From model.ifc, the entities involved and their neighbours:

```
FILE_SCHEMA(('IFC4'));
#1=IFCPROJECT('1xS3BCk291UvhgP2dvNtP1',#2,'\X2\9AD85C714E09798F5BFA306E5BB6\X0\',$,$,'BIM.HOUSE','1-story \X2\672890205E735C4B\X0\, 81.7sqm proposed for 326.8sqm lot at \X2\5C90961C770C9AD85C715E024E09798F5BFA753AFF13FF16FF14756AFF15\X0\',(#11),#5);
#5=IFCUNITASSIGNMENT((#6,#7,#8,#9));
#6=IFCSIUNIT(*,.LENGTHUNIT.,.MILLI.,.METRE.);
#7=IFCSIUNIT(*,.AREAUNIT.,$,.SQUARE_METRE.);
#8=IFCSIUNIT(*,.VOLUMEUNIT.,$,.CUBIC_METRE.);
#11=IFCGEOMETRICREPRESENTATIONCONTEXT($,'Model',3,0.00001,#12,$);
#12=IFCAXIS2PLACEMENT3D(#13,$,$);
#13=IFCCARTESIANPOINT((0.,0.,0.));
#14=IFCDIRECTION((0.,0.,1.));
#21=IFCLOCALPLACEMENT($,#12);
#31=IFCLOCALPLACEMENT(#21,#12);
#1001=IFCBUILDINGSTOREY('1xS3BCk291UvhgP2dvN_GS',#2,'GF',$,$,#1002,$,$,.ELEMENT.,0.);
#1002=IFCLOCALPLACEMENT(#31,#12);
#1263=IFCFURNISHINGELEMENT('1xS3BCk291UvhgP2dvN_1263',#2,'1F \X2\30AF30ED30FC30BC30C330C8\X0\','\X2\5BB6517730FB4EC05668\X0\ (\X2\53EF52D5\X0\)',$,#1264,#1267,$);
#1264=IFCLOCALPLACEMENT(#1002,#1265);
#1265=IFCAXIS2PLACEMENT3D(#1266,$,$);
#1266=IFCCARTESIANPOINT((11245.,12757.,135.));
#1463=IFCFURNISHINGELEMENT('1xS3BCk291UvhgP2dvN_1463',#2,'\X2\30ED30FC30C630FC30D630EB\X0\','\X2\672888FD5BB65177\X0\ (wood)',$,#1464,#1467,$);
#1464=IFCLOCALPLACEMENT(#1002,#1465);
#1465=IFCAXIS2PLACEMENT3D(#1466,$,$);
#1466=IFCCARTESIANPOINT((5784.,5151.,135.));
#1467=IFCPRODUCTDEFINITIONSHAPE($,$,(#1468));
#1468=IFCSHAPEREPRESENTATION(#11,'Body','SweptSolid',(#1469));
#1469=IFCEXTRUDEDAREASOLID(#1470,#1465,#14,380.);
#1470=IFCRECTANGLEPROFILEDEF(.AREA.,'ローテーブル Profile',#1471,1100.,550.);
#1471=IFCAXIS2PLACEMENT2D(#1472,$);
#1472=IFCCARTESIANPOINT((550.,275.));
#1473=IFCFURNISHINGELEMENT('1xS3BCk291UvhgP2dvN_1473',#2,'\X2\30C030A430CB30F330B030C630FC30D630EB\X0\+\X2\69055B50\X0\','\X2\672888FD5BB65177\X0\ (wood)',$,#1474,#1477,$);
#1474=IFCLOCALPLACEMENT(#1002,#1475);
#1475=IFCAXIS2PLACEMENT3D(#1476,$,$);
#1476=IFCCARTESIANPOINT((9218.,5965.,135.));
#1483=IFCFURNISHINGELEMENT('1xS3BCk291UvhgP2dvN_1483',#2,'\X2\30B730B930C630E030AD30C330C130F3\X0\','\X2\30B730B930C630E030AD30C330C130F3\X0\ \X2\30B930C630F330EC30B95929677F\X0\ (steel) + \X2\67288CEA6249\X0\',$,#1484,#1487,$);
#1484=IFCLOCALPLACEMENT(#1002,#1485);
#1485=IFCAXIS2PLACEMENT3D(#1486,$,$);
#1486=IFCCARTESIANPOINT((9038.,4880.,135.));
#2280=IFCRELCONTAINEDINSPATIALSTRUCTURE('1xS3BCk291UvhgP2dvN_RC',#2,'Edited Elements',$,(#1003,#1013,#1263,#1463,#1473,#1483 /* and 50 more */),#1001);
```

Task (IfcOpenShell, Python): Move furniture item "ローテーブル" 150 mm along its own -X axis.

```python
import ifcopenshell
import ifcopenshell.api.geometry
import ifcopenshell.util.placement
import ifcopenshell.util.unit

model = ifcopenshell.open("model.ifc")
unit_scale = ifcopenshell.util.unit.calculate_unit_scale(model)

item = model.by_id(1463)
matrix = ifcopenshell.util.placement.get_local_placement(item.ObjectPlacement)
matrix[:3, 3] -= matrix[:3, 0] * 0.15 / unit_scale
ifcopenshell.api.geometry.edit_object_placement(model, product=item, matrix=matrix, is_si=False)

print(ifcopenshell.util.placement.get_local_placement(item.ObjectPlacement).round(3) + 0.0)

model.write("model-out.ifc")
```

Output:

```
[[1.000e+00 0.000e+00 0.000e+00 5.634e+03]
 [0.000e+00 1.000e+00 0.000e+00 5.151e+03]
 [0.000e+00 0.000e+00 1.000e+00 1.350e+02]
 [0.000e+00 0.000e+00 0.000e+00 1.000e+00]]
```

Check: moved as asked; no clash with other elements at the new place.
